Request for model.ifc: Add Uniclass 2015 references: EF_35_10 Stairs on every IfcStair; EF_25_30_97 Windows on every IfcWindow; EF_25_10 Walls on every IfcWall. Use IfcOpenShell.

First a look at what the model holds.

```python
import ifcopenshell

model = ifcopenshell.open("model.ifc")
print(model.schema)
print("classifications:", [c.Name for c in model.by_type("IfcClassification")])
for ifc_class in ("IfcDoor", "IfcRoof", "IfcStair", "IfcWall", "IfcWindow"):
    print(ifc_class, len(model.by_type(ifc_class)))
```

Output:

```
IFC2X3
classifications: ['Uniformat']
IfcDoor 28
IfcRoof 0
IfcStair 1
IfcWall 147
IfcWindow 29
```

```python
import ifcopenshell
import ifcopenshell.api.classification

model = ifcopenshell.open("model.ifc")

# IFC2X3 requires Source and Edition and has no link from the project to the system.
system = model.create_entity("IfcClassification", Source="NBS", Edition="2015", Name="Uniclass 2015")

codes = {
    "IfcStair": ("EF_35_10", "Stairs"),
    "IfcWindow": ("EF_25_30_97", "Windows"),
    "IfcWall": ("EF_25_10", "Walls"),
}
for ifc_class, (code, name) in codes.items():
    products = model.by_type(ifc_class)
    ifcopenshell.api.classification.add_reference(
        model, products=products, classification=system, identification=code, name=name
    )
    print(code, len(products))

model.write("model-out.ifc")
```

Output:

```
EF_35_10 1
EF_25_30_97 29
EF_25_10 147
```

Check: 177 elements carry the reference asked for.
